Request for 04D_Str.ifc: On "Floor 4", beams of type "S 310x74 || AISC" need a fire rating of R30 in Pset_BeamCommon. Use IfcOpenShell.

First a look at what the model holds.

```python
import ifcopenshell
import ifcopenshell.util.element

model = ifcopenshell.open("04D_Str.ifc")
print(model.schema)
storey = next(s for s in model.by_type("IfcBuildingStorey") if s.Name == "Floor 4")
beams = [e for e in ifcopenshell.util.element.get_decomposition(storey) if e.is_a("IfcBeam")]
seen = {}
for e in beams:
    element_type = ifcopenshell.util.element.get_type(e)
    key = (element_type.Name if element_type != e and element_type else None, ifcopenshell.util.element.get_pset(e, "Pset_BeamCommon", "FireRating"))
    seen[key] = seen.get(key, 0) + 1
for (name, value), count in sorted(seen.items(), key=str):
    print(count, "x", name, "|", value)
```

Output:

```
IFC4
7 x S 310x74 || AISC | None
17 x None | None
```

```python
import ifcopenshell
import ifcopenshell.api.pset
import ifcopenshell.util.element

model = ifcopenshell.open("04D_Str.ifc")

storey = next(s for s in model.by_type("IfcBuildingStorey") if s.Name == "Floor 4")
beams = [e for e in ifcopenshell.util.element.get_decomposition(storey) if e.is_a("IfcBeam")]

count = 0
for e in beams:
    element_type = ifcopenshell.util.element.get_type(e)
    if element_type in (None, e) or element_type.Name != "S 310x74 || AISC":
        continue
    # add_pset returns the element's existing set when there is one.
    pset = ifcopenshell.api.pset.add_pset(model, product=e, name="Pset_BeamCommon")
    ifcopenshell.api.pset.edit_pset(model, pset=pset, properties={"FireRating": "R30"})
    count += 1

print(count, "beams updated")

model.write("04D_Str_updated.ifc")
```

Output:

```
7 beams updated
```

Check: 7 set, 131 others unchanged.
